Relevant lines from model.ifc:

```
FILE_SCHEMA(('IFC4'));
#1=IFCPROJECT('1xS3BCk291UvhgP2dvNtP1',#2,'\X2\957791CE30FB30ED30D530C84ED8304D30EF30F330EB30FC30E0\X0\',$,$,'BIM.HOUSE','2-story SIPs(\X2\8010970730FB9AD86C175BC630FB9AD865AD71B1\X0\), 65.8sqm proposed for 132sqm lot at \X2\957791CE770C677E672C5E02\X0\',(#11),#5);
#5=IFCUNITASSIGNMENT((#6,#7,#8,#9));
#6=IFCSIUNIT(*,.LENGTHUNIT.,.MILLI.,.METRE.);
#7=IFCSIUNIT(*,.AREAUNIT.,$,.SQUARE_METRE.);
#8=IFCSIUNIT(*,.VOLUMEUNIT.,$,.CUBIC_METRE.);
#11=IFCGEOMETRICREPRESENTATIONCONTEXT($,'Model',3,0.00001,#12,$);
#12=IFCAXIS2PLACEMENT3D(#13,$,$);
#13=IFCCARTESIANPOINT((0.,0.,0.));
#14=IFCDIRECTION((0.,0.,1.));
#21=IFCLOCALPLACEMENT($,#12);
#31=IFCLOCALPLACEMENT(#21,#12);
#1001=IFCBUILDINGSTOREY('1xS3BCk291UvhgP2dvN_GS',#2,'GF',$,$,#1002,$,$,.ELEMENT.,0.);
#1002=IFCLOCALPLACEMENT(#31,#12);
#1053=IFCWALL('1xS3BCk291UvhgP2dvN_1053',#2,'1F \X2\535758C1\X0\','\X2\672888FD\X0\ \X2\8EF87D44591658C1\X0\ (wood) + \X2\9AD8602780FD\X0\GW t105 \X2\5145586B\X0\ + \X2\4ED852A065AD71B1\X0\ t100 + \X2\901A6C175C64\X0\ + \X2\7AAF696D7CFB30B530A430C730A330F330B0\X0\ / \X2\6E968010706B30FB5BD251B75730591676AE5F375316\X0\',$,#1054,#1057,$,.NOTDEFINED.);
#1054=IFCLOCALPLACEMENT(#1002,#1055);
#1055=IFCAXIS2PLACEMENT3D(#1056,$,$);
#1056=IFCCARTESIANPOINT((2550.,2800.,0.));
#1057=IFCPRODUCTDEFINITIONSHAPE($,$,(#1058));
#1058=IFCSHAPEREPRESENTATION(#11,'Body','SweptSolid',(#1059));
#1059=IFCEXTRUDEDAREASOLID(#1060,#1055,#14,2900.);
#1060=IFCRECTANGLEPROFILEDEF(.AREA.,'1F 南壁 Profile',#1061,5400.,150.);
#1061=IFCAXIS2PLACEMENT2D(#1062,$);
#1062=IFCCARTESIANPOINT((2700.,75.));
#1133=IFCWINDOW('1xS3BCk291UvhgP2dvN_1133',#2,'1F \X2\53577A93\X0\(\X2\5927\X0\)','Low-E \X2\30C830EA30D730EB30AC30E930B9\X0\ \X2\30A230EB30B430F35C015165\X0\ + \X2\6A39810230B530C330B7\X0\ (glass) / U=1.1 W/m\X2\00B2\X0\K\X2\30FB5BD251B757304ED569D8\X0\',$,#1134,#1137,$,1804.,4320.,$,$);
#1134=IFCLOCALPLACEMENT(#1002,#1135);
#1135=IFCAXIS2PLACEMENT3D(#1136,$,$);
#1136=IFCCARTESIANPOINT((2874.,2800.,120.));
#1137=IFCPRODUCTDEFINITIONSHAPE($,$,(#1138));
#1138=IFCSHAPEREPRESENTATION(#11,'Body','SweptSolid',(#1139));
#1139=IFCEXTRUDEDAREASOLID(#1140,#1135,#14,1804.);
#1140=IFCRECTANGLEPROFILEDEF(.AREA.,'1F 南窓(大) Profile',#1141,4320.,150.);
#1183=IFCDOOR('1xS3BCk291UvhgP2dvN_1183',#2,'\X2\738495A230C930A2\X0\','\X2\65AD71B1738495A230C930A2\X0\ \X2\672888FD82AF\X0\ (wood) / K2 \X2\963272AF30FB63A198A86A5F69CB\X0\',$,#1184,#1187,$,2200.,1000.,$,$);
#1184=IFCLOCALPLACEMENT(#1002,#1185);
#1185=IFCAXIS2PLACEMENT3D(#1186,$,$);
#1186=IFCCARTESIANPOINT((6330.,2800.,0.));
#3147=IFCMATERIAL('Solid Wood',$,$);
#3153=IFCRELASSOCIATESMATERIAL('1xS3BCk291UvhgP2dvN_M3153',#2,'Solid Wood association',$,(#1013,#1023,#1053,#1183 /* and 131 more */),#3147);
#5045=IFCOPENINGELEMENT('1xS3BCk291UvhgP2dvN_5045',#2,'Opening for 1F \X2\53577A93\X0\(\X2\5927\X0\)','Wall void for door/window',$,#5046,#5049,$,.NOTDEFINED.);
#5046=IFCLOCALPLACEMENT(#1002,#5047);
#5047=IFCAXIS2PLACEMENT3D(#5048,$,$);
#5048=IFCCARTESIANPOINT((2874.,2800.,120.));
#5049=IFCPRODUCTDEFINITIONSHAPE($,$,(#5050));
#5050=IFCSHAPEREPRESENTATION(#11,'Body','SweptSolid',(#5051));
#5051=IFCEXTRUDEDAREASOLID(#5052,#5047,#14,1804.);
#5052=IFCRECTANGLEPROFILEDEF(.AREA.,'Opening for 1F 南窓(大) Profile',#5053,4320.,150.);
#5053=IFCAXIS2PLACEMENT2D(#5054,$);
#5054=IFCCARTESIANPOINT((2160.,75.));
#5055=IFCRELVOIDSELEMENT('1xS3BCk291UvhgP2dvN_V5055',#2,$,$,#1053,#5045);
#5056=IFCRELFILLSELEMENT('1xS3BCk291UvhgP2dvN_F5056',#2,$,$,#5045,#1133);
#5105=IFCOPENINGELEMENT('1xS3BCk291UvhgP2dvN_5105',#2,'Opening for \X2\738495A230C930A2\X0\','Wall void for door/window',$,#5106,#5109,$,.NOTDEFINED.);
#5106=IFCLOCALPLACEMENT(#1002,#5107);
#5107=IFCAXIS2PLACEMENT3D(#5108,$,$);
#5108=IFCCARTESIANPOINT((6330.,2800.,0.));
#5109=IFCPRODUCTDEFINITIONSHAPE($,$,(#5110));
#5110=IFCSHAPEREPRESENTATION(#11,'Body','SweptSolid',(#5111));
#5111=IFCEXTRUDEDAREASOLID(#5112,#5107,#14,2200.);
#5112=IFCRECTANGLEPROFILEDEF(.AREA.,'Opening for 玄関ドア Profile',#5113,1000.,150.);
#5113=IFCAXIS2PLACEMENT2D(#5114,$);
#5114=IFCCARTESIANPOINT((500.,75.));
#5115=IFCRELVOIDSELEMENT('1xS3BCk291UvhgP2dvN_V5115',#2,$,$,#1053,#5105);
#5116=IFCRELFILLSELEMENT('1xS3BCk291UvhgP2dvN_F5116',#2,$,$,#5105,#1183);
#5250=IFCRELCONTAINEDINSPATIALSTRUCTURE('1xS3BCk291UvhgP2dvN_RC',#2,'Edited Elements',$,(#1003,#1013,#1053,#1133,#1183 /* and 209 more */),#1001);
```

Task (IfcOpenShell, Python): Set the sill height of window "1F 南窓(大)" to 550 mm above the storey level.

```python
import numpy as np
import ifcopenshell
import ifcopenshell.api.geometry
import ifcopenshell.geom
import ifcopenshell.util.element
import ifcopenshell.util.placement
import ifcopenshell.util.shape
import ifcopenshell.util.unit

model = ifcopenshell.open("model.ifc")
unit_scale = ifcopenshell.util.unit.calculate_unit_scale(model)

window = model.by_id(1133)
opening = window.FillsVoids[0].RelatingOpeningElement
storey = ifcopenshell.util.element.get_container(window, ifc_class="IfcBuildingStorey")
level = ifcopenshell.util.placement.get_local_placement(storey.ObjectPlacement)[2, 3]

# The opening's origin need not be at the sill, so measure its lowest point.
shape = ifcopenshell.geom.create_shape(ifcopenshell.geom.settings(), opening)
bottom = ifcopenshell.util.shape.get_shape_bottom_elevation(shape, shape.geometry) / unit_scale
dz = level + 550.0 - bottom

shift = np.array([0.0, 0.0, dz])
# The window is not placed relative to its opening, so move both.
for product in (opening, window):
    matrix = ifcopenshell.util.placement.get_local_placement(product.ObjectPlacement)
    matrix[:3, 3] += shift
    ifcopenshell.api.geometry.edit_object_placement(model, product=product, matrix=matrix, is_si=False)

print(f"moved by {dz * unit_scale:+.3f} m")

model.write("model-out.ifc")
```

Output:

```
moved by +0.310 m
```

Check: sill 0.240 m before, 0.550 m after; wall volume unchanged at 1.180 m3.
